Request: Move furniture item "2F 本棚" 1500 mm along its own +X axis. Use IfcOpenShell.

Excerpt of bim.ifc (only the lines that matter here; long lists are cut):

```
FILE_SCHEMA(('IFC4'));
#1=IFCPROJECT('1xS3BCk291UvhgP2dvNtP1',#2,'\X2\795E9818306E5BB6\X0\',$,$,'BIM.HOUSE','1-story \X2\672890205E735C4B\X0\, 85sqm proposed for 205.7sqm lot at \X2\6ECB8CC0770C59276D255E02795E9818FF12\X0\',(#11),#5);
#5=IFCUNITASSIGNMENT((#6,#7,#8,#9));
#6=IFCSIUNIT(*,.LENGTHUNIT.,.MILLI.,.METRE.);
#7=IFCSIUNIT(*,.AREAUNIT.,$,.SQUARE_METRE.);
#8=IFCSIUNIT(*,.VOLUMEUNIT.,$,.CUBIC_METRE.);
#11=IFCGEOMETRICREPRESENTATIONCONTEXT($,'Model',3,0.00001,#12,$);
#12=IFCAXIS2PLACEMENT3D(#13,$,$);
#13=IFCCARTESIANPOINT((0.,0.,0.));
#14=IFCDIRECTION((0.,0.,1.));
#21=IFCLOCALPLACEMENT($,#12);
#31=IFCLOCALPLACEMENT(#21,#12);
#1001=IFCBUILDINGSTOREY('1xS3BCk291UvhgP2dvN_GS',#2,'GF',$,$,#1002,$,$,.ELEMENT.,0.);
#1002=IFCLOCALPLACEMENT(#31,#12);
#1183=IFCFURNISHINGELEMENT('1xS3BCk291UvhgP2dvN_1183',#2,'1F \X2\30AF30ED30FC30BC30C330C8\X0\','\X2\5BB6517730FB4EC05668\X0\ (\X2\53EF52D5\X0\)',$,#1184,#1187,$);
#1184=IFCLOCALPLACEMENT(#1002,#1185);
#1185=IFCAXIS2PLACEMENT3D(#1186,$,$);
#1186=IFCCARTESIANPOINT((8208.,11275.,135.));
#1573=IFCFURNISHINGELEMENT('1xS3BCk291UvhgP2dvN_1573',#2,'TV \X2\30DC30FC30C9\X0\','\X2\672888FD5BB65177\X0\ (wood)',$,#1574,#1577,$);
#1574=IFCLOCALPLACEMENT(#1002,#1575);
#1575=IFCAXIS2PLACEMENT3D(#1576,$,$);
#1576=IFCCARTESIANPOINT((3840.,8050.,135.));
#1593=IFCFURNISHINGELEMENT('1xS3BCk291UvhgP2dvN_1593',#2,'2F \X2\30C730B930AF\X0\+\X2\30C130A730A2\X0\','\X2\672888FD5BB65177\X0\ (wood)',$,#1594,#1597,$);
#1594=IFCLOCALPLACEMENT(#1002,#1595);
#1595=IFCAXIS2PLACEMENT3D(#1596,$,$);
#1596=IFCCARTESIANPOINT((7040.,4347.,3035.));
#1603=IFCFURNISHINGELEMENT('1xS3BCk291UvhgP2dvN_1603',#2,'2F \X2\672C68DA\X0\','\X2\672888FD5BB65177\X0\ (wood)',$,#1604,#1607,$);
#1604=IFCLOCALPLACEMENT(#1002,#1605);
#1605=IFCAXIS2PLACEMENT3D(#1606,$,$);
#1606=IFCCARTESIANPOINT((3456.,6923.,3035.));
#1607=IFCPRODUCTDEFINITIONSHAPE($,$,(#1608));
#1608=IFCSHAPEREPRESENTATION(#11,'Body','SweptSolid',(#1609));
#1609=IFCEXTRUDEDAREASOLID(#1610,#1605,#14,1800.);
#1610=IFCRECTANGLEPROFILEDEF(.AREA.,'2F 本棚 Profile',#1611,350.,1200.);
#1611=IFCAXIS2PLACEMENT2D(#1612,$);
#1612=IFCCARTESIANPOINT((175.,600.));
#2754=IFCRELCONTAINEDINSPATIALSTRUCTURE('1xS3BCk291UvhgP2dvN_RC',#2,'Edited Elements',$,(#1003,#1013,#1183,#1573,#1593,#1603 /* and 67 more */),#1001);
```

```python
import ifcopenshell
import ifcopenshell.api.geometry
import ifcopenshell.util.placement
import ifcopenshell.util.unit

model = ifcopenshell.open("bim.ifc")
unit_scale = ifcopenshell.util.unit.calculate_unit_scale(model)

item = model.by_id(1603)
matrix = ifcopenshell.util.placement.get_local_placement(item.ObjectPlacement)
matrix[:3, 3] += matrix[:3, 0] * 1.5 / unit_scale
ifcopenshell.api.geometry.edit_object_placement(model, product=item, matrix=matrix, is_si=False)

print(ifcopenshell.util.placement.get_local_placement(item.ObjectPlacement).round(3) + 0.0)

model.write("bim-out.ifc")
```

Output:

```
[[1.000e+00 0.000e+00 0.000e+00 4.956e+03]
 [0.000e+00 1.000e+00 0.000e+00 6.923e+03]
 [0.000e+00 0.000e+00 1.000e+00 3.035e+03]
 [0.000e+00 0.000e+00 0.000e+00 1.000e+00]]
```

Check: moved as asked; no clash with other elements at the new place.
